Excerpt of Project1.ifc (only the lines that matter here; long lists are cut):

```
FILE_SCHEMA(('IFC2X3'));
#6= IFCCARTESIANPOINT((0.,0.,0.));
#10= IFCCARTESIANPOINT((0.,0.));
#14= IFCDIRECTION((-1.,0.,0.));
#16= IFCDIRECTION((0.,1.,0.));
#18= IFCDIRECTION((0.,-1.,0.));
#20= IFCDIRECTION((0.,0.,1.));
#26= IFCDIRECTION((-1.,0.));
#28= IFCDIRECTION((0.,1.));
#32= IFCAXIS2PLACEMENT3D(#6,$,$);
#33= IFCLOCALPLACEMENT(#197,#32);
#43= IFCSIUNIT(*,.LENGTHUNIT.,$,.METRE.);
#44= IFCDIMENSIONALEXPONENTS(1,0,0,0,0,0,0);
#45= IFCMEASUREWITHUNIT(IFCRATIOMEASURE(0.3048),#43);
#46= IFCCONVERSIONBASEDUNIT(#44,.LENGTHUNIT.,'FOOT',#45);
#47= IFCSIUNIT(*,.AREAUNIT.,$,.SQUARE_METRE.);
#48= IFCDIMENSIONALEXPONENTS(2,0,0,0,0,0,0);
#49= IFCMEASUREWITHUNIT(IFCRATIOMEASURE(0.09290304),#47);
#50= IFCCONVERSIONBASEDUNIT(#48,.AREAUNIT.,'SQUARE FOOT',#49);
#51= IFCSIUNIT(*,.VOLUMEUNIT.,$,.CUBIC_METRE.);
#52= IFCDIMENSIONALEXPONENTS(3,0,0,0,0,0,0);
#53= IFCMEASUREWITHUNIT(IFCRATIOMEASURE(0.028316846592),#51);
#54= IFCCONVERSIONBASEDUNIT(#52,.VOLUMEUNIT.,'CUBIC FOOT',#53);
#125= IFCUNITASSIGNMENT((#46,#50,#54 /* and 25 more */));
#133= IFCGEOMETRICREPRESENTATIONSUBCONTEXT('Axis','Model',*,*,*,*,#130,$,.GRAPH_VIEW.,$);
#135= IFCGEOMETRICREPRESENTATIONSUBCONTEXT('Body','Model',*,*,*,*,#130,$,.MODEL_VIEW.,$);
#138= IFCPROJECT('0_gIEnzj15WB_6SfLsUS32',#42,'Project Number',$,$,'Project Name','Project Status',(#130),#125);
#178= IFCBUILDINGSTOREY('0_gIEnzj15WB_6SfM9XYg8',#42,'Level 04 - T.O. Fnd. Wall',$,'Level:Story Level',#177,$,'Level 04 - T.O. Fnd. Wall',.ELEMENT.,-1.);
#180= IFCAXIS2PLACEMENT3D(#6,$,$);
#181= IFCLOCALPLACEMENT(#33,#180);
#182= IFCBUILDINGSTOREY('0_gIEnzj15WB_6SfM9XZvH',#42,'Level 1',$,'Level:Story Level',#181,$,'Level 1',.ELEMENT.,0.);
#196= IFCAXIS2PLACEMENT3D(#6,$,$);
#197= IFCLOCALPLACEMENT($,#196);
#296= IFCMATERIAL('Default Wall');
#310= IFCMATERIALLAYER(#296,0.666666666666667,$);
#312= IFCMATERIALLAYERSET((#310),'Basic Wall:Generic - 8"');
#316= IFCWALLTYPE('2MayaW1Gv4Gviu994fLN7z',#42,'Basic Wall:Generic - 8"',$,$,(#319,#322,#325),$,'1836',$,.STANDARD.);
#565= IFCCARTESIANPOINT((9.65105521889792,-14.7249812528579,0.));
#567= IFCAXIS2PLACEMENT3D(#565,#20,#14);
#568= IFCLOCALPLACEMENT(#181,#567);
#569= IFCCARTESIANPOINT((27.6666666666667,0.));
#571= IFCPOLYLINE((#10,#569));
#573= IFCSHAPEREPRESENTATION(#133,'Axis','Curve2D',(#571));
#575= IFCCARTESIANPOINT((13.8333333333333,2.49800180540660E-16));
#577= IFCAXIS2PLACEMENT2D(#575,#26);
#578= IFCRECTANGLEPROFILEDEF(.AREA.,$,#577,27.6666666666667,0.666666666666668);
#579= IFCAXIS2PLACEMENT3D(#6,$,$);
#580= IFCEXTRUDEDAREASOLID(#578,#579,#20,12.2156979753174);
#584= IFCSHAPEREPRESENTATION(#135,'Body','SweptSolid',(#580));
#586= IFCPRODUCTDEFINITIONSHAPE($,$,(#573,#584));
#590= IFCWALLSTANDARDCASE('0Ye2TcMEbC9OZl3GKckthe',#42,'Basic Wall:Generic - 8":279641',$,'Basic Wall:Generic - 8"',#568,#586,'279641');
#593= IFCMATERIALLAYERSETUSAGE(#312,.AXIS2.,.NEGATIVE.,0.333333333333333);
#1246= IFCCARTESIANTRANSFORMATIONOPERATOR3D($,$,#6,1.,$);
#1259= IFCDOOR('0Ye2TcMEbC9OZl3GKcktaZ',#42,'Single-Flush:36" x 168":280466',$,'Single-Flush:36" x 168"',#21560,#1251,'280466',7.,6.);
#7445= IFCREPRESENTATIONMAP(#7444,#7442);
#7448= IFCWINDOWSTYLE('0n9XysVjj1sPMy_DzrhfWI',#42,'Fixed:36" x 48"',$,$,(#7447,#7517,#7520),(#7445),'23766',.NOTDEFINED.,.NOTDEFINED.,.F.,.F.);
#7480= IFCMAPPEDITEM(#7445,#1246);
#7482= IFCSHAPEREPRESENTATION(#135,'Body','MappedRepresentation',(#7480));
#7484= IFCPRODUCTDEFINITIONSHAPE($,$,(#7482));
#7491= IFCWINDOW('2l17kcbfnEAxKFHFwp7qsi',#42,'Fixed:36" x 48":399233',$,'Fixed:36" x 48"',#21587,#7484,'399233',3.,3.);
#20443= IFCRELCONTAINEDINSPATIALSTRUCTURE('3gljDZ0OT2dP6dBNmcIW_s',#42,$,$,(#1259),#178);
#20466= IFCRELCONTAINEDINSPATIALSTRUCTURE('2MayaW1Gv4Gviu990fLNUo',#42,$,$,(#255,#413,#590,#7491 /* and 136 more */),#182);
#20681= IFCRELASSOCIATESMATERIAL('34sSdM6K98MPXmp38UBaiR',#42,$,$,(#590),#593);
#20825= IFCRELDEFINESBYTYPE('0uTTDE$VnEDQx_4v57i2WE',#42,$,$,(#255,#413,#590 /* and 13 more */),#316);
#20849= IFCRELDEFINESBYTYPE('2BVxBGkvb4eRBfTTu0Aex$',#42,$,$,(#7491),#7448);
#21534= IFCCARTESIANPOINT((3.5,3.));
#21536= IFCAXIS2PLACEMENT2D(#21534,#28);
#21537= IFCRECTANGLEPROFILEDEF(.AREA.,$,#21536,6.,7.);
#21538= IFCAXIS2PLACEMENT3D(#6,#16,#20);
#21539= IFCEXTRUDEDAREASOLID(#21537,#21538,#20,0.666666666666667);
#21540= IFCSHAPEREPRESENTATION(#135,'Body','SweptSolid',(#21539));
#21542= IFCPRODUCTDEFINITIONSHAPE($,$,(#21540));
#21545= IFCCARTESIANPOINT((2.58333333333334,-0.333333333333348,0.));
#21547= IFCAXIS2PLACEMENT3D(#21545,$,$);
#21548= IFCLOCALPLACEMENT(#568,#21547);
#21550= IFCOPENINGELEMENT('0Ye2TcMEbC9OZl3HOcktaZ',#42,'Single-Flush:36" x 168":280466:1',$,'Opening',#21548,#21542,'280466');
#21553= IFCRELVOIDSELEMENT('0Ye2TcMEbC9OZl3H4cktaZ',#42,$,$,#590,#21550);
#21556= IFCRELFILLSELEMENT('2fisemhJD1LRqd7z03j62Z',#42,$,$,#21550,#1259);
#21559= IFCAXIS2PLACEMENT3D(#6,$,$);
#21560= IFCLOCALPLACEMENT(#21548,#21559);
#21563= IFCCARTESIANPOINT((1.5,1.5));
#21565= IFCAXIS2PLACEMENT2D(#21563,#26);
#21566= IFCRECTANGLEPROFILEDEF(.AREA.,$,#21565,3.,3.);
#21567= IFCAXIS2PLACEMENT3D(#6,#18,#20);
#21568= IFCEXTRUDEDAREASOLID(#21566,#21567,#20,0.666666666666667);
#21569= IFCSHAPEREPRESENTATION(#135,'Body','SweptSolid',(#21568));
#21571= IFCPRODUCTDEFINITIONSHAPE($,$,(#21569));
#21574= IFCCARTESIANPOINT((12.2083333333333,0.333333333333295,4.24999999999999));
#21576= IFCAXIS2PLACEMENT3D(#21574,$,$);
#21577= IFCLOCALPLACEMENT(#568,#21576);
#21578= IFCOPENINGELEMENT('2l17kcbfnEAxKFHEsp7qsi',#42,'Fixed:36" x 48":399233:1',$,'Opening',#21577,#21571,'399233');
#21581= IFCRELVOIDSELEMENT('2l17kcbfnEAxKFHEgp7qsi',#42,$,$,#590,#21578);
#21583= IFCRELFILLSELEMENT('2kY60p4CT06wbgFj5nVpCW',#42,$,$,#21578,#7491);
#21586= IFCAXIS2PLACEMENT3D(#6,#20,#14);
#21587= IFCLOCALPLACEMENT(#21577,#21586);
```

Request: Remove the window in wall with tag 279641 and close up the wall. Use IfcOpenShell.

```python
import ifcopenshell
import ifcopenshell.api.feature
import ifcopenshell.api.root
import ifcopenshell.geom
import ifcopenshell.util.shape

model = ifcopenshell.open("Project1.ifc")
settings = ifcopenshell.geom.settings()


def volume(element):
    """Net volume in cubic metres, openings subtracted."""
    shape = ifcopenshell.geom.create_shape(settings, element)
    return ifcopenshell.util.shape.get_volume(shape.geometry)


window = model.by_guid("2l17kcbfnEAxKFHFwp7qsi")
opening = window.FillsVoids[0].RelatingOpeningElement
wall = opening.VoidsElements[0].RelatingBuildingElement
before = volume(wall)

ifcopenshell.api.root.remove_product(model, product=window)
ifcopenshell.api.feature.remove_feature(model, feature=opening)

after = volume(wall)

print(f"wall volume {before:.3f} -> {after:.3f} m3")

model.write("Project1_v2.ifc")
```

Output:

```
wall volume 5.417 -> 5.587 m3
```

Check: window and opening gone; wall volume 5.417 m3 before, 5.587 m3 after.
